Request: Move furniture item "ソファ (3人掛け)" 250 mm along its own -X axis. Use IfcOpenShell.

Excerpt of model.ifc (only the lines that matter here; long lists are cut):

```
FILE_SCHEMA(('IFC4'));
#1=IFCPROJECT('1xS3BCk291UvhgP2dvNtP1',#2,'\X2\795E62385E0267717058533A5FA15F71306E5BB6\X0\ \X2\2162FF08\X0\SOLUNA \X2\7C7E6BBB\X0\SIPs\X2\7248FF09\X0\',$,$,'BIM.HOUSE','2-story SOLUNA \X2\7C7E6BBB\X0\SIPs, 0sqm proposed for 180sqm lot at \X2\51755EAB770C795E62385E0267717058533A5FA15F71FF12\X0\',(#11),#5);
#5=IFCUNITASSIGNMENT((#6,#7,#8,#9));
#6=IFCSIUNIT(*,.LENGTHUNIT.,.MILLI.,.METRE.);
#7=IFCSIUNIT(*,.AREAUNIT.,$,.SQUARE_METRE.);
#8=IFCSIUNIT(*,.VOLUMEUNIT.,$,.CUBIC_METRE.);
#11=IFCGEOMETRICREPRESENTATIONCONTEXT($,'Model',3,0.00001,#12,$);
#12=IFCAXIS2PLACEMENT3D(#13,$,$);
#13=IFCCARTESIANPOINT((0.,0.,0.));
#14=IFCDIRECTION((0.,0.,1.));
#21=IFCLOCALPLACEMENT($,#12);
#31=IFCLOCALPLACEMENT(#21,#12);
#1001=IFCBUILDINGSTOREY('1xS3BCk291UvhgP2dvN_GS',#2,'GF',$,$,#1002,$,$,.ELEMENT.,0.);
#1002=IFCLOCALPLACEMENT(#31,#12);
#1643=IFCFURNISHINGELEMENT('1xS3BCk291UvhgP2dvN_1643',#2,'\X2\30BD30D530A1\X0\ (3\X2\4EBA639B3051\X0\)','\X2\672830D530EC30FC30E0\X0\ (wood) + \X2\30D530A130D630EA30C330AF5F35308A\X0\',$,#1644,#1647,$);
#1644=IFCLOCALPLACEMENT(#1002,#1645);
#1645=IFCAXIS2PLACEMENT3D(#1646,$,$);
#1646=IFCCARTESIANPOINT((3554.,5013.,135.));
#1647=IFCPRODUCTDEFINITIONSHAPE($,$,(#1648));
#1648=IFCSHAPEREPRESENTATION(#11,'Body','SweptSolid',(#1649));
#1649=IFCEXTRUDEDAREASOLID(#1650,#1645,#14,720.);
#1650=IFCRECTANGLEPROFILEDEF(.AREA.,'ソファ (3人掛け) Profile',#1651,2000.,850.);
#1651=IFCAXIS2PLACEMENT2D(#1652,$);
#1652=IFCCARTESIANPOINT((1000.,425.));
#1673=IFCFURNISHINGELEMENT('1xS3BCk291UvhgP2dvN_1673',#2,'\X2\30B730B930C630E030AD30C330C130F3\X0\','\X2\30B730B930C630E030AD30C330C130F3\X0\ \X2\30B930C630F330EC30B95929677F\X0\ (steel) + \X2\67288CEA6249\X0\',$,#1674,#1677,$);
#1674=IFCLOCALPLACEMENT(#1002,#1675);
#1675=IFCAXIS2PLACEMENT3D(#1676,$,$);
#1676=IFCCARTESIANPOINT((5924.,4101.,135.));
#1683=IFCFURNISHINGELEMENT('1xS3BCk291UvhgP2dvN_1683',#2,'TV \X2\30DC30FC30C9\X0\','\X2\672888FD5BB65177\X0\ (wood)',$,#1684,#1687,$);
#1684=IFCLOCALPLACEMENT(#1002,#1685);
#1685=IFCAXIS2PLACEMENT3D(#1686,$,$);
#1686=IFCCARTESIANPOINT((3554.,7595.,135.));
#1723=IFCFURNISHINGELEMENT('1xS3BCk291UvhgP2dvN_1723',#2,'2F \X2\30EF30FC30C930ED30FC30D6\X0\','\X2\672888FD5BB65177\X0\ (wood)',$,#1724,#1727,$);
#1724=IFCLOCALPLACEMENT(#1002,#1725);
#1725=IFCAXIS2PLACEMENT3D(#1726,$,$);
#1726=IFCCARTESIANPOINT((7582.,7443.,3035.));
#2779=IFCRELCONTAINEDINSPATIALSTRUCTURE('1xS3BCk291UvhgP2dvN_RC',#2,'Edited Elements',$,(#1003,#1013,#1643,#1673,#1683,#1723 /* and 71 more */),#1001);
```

```python
import ifcopenshell
import ifcopenshell.api.geometry
import ifcopenshell.util.placement

model = ifcopenshell.open("model.ifc")

item = model.by_id(1643)
matrix = ifcopenshell.util.placement.get_local_placement(item.ObjectPlacement)
matrix[:3, 3] -= matrix[:3, 0] * 250.0
ifcopenshell.api.geometry.edit_object_placement(model, product=item, matrix=matrix, is_si=False)

print(ifcopenshell.util.placement.get_local_placement(item.ObjectPlacement).round(3) + 0.0)

model.write("model_updated.ifc")
```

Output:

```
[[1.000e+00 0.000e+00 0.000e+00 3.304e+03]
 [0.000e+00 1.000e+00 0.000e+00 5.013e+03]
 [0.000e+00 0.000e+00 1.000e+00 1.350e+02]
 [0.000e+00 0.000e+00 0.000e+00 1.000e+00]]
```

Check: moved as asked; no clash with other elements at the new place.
